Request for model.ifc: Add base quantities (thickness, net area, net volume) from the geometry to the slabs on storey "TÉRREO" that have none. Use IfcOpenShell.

First a look at what the model holds.

```python
import ifcopenshell
import ifcopenshell.util.element
import ifcopenshell.util.unit

model = ifcopenshell.open("model.ifc")
print(model.schema)
for unit_type in ("LENGTHUNIT", "AREAUNIT", "VOLUMEUNIT"):
    print(unit_type, ifcopenshell.util.unit.calculate_unit_scale(model, unit_type))
storey = next(s for s in model.by_type("IfcBuildingStorey") if s.Name == "TÉRREO")
slabs = [e for e in ifcopenshell.util.element.get_decomposition(storey) if e.is_a("IfcSlab")]
for e in sorted(slabs, key=lambda e: e.id()):
    print(e.id(), e.is_a(), e.Name, list(ifcopenshell.util.element.get_psets(e, qtos_only=True)), sep=" | ")
```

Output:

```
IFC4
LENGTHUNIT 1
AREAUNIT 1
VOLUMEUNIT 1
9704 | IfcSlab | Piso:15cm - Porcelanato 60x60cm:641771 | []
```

```python
import ifcopenshell
import ifcopenshell.api.pset
import ifcopenshell.geom
import ifcopenshell.util.element
import ifcopenshell.util.shape
import ifcopenshell.util.unit

model = ifcopenshell.open("model.ifc")
unit_scale = ifcopenshell.util.unit.calculate_unit_scale(model)
area_scale = ifcopenshell.util.unit.calculate_unit_scale(model, "AREAUNIT")
volume_scale = ifcopenshell.util.unit.calculate_unit_scale(model, "VOLUMEUNIT")
settings = ifcopenshell.geom.settings()

storey = next(s for s in model.by_type("IfcBuildingStorey") if s.Name == "TÉRREO")
slabs = [e for e in ifcopenshell.util.element.get_decomposition(storey) if e.is_a("IfcSlab")]

for e in sorted(slabs, key=lambda e: e.id()):
    if ifcopenshell.util.element.get_psets(e, qtos_only=True, should_inherit=False):
        continue
    # Geometry comes back in metres, in the element's own axes.
    shape = ifcopenshell.geom.create_shape(settings, e)
    values = {
        "Width": ifcopenshell.util.shape.get_z(shape.geometry) / unit_scale,
        "NetArea": ifcopenshell.util.shape.get_footprint_area(shape.geometry) / area_scale,
        "NetVolume": ifcopenshell.util.shape.get_volume(shape.geometry) / volume_scale,
    }
    qto = ifcopenshell.api.pset.add_qto(model, product=e, name="Qto_SlabBaseQuantities")
    ifcopenshell.api.pset.edit_qto(model, qto=qto, properties=values)
    print(e.id(), {k: round(v, 3) for k, v in values.items()})

model.write("model_updated.ifc")
```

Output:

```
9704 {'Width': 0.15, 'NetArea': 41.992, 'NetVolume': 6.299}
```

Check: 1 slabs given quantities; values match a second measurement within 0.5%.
